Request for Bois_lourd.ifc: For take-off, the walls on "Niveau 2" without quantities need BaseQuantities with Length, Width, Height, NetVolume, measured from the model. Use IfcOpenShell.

First a look at what the model holds.

```python
import ifcopenshell
import ifcopenshell.util.element
import ifcopenshell.util.unit

model = ifcopenshell.open("Bois_lourd.ifc")
print(model.schema)
for unit_type in ("LENGTHUNIT", "AREAUNIT", "VOLUMEUNIT"):
    print(unit_type, ifcopenshell.util.unit.calculate_unit_scale(model, unit_type))
storey = next(s for s in model.by_type("IfcBuildingStorey") if s.Name == "Niveau 2")
walls = [e for e in ifcopenshell.util.element.get_decomposition(storey) if e.is_a("IfcWall")]
for e in sorted(walls, key=lambda e: e.id()):
    print(e.id(), e.is_a(), e.Name, list(ifcopenshell.util.element.get_psets(e, qtos_only=True)), sep=" | ")
```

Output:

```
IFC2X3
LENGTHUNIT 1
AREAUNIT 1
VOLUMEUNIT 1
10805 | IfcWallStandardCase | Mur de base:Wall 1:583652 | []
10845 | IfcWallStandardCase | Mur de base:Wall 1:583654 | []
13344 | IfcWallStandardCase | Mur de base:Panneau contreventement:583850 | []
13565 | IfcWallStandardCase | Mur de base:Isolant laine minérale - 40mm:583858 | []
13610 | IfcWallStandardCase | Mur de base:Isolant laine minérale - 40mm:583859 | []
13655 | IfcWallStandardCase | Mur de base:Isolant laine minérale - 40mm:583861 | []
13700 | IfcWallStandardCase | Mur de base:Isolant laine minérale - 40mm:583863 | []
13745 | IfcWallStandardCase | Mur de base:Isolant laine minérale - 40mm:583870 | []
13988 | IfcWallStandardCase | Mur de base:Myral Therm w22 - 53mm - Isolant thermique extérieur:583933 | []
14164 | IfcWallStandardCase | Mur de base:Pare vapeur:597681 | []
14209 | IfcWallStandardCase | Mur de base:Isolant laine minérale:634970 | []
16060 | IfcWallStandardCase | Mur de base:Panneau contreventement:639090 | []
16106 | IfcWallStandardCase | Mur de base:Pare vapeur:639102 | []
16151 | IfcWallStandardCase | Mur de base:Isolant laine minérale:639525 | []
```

```python
import ifcopenshell
import ifcopenshell.api.pset
import ifcopenshell.geom
import ifcopenshell.util.element
import ifcopenshell.util.shape
import ifcopenshell.util.unit

model = ifcopenshell.open("Bois_lourd.ifc")
unit_scale = ifcopenshell.util.unit.calculate_unit_scale(model)
volume_scale = ifcopenshell.util.unit.calculate_unit_scale(model, "VOLUMEUNIT")
settings = ifcopenshell.geom.settings()

storey = next(s for s in model.by_type("IfcBuildingStorey") if s.Name == "Niveau 2")
walls = [e for e in ifcopenshell.util.element.get_decomposition(storey) if e.is_a("IfcWall")]

for e in sorted(walls, key=lambda e: e.id()):
    if ifcopenshell.util.element.get_psets(e, qtos_only=True, should_inherit=False):
        continue
    # Geometry comes back in metres, in the element's own axes.
    shape = ifcopenshell.geom.create_shape(settings, e)
    values = {
        "Length": ifcopenshell.util.shape.get_x(shape.geometry) / unit_scale,
        "Width": ifcopenshell.util.shape.get_y(shape.geometry) / unit_scale,
        "Height": ifcopenshell.util.shape.get_z(shape.geometry) / unit_scale,
        "NetVolume": ifcopenshell.util.shape.get_volume(shape.geometry) / volume_scale,
    }
    qto = ifcopenshell.api.pset.add_qto(model, product=e, name="BaseQuantities")
    ifcopenshell.api.pset.edit_qto(model, qto=qto, properties=values)
    print(e.id(), {k: round(v, 3) for k, v in values.items()})

model.write("Bois_lourd_edited.ifc")
```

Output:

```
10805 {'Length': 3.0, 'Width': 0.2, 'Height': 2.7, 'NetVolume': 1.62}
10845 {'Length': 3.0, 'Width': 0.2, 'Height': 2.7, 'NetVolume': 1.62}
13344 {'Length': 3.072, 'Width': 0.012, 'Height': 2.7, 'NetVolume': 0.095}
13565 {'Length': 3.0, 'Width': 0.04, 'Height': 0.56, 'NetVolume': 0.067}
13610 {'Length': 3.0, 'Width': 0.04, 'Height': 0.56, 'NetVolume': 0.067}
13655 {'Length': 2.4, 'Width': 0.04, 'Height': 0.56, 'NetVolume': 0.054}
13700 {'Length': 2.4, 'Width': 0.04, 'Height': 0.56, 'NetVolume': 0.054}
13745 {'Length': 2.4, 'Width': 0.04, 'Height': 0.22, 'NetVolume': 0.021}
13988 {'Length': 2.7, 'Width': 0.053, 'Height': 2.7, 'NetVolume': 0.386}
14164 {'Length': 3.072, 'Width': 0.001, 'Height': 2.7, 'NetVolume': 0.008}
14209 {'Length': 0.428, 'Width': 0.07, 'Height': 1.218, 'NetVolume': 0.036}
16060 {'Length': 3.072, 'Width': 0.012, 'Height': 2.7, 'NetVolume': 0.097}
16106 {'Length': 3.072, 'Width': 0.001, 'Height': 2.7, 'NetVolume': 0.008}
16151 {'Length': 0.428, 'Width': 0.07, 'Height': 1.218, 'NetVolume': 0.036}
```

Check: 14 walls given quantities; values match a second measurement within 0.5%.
